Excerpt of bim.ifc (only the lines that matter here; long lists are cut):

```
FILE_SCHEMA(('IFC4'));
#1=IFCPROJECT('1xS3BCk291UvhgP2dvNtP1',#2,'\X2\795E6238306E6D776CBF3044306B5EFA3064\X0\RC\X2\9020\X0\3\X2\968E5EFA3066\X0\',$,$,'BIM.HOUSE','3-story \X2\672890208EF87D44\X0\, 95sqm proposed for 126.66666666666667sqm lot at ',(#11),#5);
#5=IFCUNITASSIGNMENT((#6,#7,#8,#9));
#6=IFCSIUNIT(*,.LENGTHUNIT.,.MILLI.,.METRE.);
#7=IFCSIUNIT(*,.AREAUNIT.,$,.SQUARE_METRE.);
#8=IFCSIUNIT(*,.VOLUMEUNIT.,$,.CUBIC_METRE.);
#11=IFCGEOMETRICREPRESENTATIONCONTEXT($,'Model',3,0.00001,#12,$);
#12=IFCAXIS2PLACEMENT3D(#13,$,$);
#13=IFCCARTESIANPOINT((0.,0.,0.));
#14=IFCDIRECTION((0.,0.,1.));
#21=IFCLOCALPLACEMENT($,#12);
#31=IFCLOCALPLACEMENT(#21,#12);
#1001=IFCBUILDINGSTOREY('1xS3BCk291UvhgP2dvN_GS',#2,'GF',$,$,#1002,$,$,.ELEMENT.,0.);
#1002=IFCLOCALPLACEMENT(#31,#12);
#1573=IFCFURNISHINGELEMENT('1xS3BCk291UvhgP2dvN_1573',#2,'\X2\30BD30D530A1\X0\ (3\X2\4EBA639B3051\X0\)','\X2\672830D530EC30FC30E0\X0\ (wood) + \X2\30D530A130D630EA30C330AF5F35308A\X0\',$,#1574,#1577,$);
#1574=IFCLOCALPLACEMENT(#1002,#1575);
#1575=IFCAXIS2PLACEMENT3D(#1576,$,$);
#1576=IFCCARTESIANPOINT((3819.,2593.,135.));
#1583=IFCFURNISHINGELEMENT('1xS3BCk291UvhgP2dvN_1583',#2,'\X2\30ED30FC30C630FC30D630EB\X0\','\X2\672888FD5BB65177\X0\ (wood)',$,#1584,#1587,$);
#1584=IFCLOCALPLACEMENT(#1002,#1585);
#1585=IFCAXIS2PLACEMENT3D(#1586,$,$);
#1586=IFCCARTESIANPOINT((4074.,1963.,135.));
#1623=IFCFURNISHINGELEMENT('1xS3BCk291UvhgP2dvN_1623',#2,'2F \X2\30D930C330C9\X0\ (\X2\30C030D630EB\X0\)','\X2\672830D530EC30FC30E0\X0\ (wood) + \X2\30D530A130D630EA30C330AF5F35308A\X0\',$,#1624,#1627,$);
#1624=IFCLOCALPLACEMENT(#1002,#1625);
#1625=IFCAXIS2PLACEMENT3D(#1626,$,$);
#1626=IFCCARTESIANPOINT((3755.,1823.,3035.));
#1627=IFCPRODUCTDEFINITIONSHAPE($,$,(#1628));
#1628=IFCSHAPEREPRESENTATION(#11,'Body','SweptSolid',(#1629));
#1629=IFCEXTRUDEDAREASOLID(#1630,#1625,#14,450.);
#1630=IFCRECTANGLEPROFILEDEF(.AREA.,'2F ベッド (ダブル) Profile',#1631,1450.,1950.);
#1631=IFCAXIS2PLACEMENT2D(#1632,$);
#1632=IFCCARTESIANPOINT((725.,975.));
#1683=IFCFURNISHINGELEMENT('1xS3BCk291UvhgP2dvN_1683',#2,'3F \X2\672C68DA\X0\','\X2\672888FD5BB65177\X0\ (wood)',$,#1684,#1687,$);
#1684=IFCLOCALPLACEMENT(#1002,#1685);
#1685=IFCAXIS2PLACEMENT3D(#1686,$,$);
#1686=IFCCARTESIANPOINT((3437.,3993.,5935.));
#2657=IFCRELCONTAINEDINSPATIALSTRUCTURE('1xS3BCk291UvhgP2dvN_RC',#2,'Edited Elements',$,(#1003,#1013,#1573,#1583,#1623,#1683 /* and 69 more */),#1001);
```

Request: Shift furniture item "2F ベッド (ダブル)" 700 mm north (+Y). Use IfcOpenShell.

```python
import ifcopenshell
import ifcopenshell.api.geometry
import ifcopenshell.util.placement
import ifcopenshell.util.unit

model = ifcopenshell.open("bim.ifc")
unit_scale = ifcopenshell.util.unit.calculate_unit_scale(model)

item = model.by_guid("1xS3BCk291UvhgP2dvN_1623")
matrix = ifcopenshell.util.placement.get_local_placement(item.ObjectPlacement)
matrix[1, 3] += 0.7 / unit_scale
ifcopenshell.api.geometry.edit_object_placement(model, product=item, matrix=matrix, is_si=False)

print(ifcopenshell.util.placement.get_local_placement(item.ObjectPlacement).round(3) + 0.0)

model.write("bim_v2.ifc")
```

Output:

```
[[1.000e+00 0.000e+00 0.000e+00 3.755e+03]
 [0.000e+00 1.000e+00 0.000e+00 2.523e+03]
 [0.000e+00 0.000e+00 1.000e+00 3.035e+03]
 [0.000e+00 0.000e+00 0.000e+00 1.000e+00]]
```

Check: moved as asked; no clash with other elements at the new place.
